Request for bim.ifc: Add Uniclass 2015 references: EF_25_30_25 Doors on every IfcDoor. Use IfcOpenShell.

First a look at what the model holds.

```python
import ifcopenshell

model = ifcopenshell.open("bim.ifc")
print(model.schema)
print("classifications:", [c.Name for c in model.by_type("IfcClassification")])
for ifc_class in ("IfcDoor", "IfcRoof", "IfcStair", "IfcWall", "IfcWindow"):
    print(ifc_class, len(model.by_type(ifc_class)))
```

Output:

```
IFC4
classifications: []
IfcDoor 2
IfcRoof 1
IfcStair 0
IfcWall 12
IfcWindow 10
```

```python
import ifcopenshell
import ifcopenshell.api.classification

model = ifcopenshell.open("bim.ifc")

system = ifcopenshell.api.classification.add_classification(model, classification="Uniclass 2015")

codes = {
    "IfcDoor": ("EF_25_30_25", "Doors"),
}
for ifc_class, (code, name) in codes.items():
    products = model.by_type(ifc_class)
    ifcopenshell.api.classification.add_reference(
        model, products=products, classification=system, identification=code, name=name
    )
    print(code, len(products))

model.write("bim-out.ifc")
```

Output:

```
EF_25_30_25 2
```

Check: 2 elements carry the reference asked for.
